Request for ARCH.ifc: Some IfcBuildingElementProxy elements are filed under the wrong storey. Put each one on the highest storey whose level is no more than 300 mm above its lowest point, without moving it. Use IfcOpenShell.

First a look at what the model holds.

```python
import ifcopenshell
import ifcopenshell.util.element
import ifcopenshell.util.placement

model = ifcopenshell.open("ARCH.ifc")
print(model.schema)
for storey in model.by_type("IfcBuildingStorey"):
    level = ifcopenshell.util.placement.get_storey_elevation(storey)
    count = sum(e.is_a("IfcBuildingElementProxy") for e in ifcopenshell.util.element.get_contained(storey))
    print(storey.id(), storey.Name, round(level, 3), count, sep=" | ")
```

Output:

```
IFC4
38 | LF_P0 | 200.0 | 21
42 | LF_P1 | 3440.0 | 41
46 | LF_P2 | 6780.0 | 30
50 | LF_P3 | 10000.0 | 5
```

```python
import ifcopenshell
import ifcopenshell.api.spatial
import ifcopenshell.geom
import ifcopenshell.util.element
import ifcopenshell.util.placement
import ifcopenshell.util.shape
import ifcopenshell.util.unit

model = ifcopenshell.open("ARCH.ifc")
unit_scale = ifcopenshell.util.unit.calculate_unit_scale(model)
settings = ifcopenshell.geom.settings()

levels = sorted(
    ((ifcopenshell.util.placement.get_storey_elevation(s) * unit_scale, s) for s in model.by_type("IfcBuildingStorey")),
    key=lambda pair: pair[0],
)

for e in model.by_type("IfcBuildingElementProxy"):
    current = e.ContainedInStructure[0].RelatingStructure if e.ContainedInStructure else None
    if current is None or not current.is_a("IfcBuildingStorey"):
        continue
    shape = ifcopenshell.geom.create_shape(settings, e)
    bottom = ifcopenshell.util.shape.get_shape_bottom_elevation(shape, shape.geometry)
    below = [s for level, s in levels if level <= bottom + 0.3]
    storey = below[-1] if below else levels[0][1]
    if storey != current:
        # assign_container keeps the world position.
        ifcopenshell.api.spatial.assign_container(model, products=[e], relating_structure=storey)
        print(e.id(), current.Name, "->", storey.Name)

model.write("ARCH_updated.ifc")
```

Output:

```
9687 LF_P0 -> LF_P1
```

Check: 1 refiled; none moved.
